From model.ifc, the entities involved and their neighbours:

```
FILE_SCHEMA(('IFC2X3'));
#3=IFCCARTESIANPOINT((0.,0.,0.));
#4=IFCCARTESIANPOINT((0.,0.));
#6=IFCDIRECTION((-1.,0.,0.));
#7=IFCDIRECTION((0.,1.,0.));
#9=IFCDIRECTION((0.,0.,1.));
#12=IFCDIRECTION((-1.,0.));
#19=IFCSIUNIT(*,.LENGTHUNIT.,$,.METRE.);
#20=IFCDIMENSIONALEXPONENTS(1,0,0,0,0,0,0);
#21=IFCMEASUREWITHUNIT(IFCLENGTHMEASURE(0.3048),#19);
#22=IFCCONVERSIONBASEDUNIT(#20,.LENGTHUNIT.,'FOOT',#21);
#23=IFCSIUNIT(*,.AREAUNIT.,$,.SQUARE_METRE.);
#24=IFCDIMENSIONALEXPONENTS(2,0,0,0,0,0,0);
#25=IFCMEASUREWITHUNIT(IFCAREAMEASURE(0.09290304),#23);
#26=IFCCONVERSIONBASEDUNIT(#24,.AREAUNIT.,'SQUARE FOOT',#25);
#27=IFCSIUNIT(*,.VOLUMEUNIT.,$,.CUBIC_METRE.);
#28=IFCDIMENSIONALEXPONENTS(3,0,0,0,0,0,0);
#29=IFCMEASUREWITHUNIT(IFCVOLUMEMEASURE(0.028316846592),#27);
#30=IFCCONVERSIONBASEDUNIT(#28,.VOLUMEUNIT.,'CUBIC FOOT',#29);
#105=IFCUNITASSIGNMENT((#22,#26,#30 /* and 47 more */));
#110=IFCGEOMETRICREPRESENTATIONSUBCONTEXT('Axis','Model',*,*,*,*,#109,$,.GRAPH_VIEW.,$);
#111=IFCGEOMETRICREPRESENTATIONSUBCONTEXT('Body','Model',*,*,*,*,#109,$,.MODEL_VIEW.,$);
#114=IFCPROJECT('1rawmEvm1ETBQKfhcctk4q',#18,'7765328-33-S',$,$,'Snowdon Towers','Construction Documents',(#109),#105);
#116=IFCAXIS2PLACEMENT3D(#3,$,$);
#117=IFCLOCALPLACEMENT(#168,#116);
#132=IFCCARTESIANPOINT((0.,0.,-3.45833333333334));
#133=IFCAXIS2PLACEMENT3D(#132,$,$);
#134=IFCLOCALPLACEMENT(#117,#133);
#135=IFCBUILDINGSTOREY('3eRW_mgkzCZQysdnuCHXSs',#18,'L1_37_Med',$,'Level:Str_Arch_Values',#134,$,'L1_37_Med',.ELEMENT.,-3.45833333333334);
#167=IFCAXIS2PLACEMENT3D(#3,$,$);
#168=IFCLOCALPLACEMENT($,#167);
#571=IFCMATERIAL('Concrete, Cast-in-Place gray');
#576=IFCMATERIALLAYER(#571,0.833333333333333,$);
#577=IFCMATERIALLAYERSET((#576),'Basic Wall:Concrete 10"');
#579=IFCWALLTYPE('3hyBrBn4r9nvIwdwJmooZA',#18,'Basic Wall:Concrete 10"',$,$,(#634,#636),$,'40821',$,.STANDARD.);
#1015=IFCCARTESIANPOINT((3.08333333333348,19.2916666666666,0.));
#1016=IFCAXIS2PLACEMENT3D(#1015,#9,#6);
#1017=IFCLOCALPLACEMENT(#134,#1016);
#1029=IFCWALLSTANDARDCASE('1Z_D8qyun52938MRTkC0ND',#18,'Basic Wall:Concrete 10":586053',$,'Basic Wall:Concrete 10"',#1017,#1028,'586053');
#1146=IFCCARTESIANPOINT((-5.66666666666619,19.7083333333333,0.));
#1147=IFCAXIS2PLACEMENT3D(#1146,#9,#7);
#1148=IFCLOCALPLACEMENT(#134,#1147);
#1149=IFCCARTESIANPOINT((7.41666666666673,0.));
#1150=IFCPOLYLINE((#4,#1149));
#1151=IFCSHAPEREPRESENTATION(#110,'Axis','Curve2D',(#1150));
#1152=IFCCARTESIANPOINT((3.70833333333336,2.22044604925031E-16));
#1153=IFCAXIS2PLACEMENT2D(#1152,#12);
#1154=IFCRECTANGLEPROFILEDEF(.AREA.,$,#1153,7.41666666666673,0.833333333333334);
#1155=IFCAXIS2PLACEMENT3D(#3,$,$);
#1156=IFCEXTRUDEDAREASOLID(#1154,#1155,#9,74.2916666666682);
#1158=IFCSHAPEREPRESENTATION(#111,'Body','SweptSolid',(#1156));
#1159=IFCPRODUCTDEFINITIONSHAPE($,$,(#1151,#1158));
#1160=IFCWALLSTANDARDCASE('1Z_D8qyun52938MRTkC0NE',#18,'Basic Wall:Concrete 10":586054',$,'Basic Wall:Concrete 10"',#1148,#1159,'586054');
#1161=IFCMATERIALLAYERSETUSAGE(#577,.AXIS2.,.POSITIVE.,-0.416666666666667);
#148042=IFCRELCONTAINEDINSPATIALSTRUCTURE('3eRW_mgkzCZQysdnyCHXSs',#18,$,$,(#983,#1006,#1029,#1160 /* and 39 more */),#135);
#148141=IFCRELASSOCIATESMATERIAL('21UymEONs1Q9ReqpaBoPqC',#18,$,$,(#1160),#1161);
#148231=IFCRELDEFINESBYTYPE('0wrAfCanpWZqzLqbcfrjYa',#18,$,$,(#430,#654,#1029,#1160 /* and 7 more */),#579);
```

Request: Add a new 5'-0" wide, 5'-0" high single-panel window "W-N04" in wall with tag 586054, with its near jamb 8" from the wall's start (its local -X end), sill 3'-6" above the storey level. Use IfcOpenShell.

```python
import numpy as np
import ifcopenshell
import ifcopenshell.api.feature
import ifcopenshell.api.geometry
import ifcopenshell.api.root
import ifcopenshell.api.spatial
import ifcopenshell.api.type
import ifcopenshell.geom
import ifcopenshell.util.element
import ifcopenshell.util.placement
import ifcopenshell.util.representation
import ifcopenshell.util.shape
import ifcopenshell.util.unit

model = ifcopenshell.open("model.ifc")
unit_scale = ifcopenshell.util.unit.calculate_unit_scale(model)
settings = ifcopenshell.geom.settings()


def volume(element):
    """Net volume in cubic metres, openings subtracted."""
    shape = ifcopenshell.geom.create_shape(settings, element)
    return ifcopenshell.util.shape.get_volume(shape.geometry)


wall = model.by_guid("1Z_D8qyun52938MRTkC0NE")
storey = ifcopenshell.util.element.get_container(wall, ifc_class="IfcBuildingStorey")
context = ifcopenshell.util.representation.get_context(model, "Model", "Body", "MODEL_VIEW")
before = volume(wall)

width, height, from_end, sill = 1.524, 1.524, 0.2032, 1.0668  # metres

# The wall runs along its own X axis, and the end named is its -X end.
wall_shape = ifcopenshell.geom.create_shape(settings, wall)
x, y, z = ifcopenshell.util.shape.get_vertices(wall_shape.geometry).T
start = x.min() + from_end
face, thickness = float(y.min()), float(y.max() - y.min())
wall_matrix = ifcopenshell.util.placement.get_local_placement(wall.ObjectPlacement)
level = ifcopenshell.util.placement.get_local_placement(storey.ObjectPlacement)[2, 3]


def in_wall(x, y):
    """Placement at x, y metres in the wall's axes, at sill height."""
    matrix = wall_matrix.copy()
    matrix[:, 3] = wall_matrix @ np.array([x / unit_scale, y / unit_scale, 0.0, 1.0])
    matrix[2, 3] = level + sill / unit_scale
    return matrix


# Opening: a box that overshoots both wall faces by 50 mm.
opening = ifcopenshell.api.root.create_entity(model, ifc_class="IfcOpeningElement")
box = ifcopenshell.api.geometry.add_wall_representation(
    model, context=context, length=width, height=height, thickness=thickness + 0.1
)
ifcopenshell.api.geometry.assign_representation(model, product=opening, representation=box)
ifcopenshell.api.geometry.edit_object_placement(model, product=opening, matrix=in_wall(start, face - 0.05), is_si=False)
ifcopenshell.api.feature.add_feature(model, feature=opening, element=wall)

window = ifcopenshell.api.root.create_entity(model, ifc_class="IfcWindow", name="W-N04")
window.OverallWidth, window.OverallHeight = width / unit_scale, height / unit_scale
body = ifcopenshell.api.geometry.add_window_representation(
    model,
    context=context,
    overall_width=window.OverallWidth,
    overall_height=window.OverallHeight,
    partition_type="SINGLE_PANEL",
)
ifcopenshell.api.geometry.assign_representation(model, product=window, representation=body)
ifcopenshell.api.spatial.assign_container(model, products=[window], relating_structure=storey)
fills = ifcopenshell.api.feature.add_filling(model, opening=opening, element=window)
fills.OwnerHistory = window.OwnerHistory  # required in IFC2X3

# IFC2X3 keeps the operation on the window style.
style = ifcopenshell.api.root.create_entity(model, ifc_class="IfcWindowStyle", name="W-N04")
style.OperationType, style.ConstructionType = "SINGLE_PANEL", "NOTDEFINED"
style.ParameterTakesPrecedence = style.Sizeable = False
ifcopenshell.api.type.assign_type(model, related_objects=[window], relating_type=style)

# Centre the window in the wall's thickness.
ifcopenshell.api.geometry.edit_object_placement(model, product=window, matrix=in_wall(start, face), is_si=False)
window_shape = ifcopenshell.geom.create_shape(settings, window)
depth = ifcopenshell.util.shape.get_vertices(window_shape.geometry)[:, 1]
offset = face + thickness / 2 - (depth.min() + depth.max()) / 2
ifcopenshell.api.geometry.edit_object_placement(model, product=window, matrix=in_wall(start, offset), is_si=False)

after = volume(wall)

print(f"wall volume {before:.3f} -> {after:.3f} m3")

model.write("model_v2.ifc")
```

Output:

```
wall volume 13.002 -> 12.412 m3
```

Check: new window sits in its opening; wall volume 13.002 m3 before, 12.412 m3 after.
